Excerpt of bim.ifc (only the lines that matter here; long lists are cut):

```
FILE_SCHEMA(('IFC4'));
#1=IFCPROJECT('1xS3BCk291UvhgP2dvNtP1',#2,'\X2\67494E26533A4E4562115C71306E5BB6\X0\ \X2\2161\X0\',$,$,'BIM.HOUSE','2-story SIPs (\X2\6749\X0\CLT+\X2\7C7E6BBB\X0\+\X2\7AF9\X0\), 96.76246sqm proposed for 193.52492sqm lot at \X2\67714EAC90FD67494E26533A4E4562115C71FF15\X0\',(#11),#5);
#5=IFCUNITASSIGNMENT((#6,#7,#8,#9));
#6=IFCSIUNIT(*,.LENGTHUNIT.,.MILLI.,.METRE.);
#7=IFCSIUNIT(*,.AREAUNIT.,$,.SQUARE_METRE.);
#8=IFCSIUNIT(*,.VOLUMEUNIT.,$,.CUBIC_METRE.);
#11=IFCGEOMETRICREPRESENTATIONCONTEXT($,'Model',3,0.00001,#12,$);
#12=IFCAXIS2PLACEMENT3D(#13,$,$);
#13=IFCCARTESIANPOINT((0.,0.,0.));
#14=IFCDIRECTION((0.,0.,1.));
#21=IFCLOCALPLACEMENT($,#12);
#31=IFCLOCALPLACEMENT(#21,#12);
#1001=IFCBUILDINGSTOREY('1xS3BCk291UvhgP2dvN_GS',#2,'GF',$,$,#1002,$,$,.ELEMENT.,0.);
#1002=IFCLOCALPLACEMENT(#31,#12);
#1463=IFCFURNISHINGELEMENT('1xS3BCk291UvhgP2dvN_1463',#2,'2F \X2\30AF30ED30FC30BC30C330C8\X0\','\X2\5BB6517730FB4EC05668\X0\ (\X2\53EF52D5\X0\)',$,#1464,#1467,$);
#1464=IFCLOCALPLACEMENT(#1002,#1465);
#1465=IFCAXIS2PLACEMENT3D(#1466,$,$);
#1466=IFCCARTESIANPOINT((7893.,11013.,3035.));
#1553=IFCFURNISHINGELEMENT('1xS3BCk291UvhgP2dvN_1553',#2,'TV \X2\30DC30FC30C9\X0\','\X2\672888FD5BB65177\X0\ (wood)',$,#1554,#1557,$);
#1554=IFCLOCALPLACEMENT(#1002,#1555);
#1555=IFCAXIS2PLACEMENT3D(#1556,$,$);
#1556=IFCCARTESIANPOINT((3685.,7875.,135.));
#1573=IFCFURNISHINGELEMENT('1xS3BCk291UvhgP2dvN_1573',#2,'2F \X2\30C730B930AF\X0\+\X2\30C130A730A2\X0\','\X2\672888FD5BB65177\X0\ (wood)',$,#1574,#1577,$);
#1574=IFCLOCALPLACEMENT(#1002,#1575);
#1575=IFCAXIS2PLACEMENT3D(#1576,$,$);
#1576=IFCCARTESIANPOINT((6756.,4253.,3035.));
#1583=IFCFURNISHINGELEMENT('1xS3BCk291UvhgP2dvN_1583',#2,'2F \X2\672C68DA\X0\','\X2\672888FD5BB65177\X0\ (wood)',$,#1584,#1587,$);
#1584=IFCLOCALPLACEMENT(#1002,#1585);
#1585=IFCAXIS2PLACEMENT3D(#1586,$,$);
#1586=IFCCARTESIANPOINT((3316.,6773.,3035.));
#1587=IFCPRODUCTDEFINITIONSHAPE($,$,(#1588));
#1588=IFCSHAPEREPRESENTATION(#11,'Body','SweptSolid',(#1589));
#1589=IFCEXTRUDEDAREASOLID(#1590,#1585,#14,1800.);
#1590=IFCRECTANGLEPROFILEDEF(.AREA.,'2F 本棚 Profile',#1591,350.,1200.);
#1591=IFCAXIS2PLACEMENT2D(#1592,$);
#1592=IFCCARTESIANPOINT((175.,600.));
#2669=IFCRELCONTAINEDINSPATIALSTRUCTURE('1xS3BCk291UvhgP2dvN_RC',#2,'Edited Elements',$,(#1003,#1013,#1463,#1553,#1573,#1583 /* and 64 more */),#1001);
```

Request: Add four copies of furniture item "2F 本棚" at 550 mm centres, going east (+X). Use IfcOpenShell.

```python
import numpy as np
import ifcopenshell
import ifcopenshell.api.geometry
import ifcopenshell.api.root
import ifcopenshell.util.element
import ifcopenshell.util.placement
import ifcopenshell.util.unit

model = ifcopenshell.open("bim.ifc")
unit_scale = ifcopenshell.util.unit.calculate_unit_scale(model)


def reuse_history(source, copy):
    """copy_class also copies each property set's owner history, people and application; keep the originals."""
    for rel in copy.IsDefinedBy:
        if rel.is_a("IfcRelDefinesByProperties") and (history := rel.RelatingPropertyDefinition.OwnerHistory):
            rel.RelatingPropertyDefinition.OwnerHistory = source.OwnerHistory
            ifcopenshell.util.element.remove_deep2(model, history)


source = model.by_guid("1xS3BCk291UvhgP2dvN_1583")
base = ifcopenshell.util.placement.get_local_placement(source.ObjectPlacement)
step = np.array([1.0, 0.0, 0.0]) * 0.55 / unit_scale

for i in range(1, 5):
    copy = ifcopenshell.api.root.copy_class(model, product=source)
    copy.Representation = ifcopenshell.util.element.copy_deep(
        model, source.Representation, exclude=["IfcGeometricRepresentationContext", "IfcRepresentationMap"]
    )
    reuse_history(source, copy)
    matrix = base.copy()
    matrix[:3, 3] += i * step
    print("added at", matrix[:3, 3].round(3) + 0.0)
    ifcopenshell.api.geometry.edit_object_placement(model, product=copy, matrix=matrix, is_si=False)

model.write("bim_edited.ifc")
```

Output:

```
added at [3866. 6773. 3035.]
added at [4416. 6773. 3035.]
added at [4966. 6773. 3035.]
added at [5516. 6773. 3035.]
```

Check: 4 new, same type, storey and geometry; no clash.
